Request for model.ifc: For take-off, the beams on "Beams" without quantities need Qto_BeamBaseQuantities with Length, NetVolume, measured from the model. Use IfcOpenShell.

First a look at what the model holds.

```python
import ifcopenshell
import ifcopenshell.util.element
import ifcopenshell.util.unit

model = ifcopenshell.open("model.ifc")
print(model.schema)
for unit_type in ("LENGTHUNIT", "AREAUNIT", "VOLUMEUNIT"):
    print(unit_type, ifcopenshell.util.unit.calculate_unit_scale(model, unit_type))
storey = next(s for s in model.by_type("IfcBuildingStorey") if s.Name == "Beams")
beams = [e for e in ifcopenshell.util.element.get_decomposition(storey) if e.is_a("IfcBeam")]
for e in sorted(beams, key=lambda e: e.id()):
    print(e.id(), e.is_a(), e.Name, list(ifcopenshell.util.element.get_psets(e, qtos_only=True)), sep=" | ")
```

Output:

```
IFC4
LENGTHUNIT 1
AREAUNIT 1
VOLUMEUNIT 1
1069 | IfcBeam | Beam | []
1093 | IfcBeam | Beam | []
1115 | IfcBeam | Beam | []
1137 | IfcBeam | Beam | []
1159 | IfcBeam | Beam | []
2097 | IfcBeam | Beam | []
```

```python
import ifcopenshell
import ifcopenshell.api.pset
import ifcopenshell.geom
import ifcopenshell.util.element
import ifcopenshell.util.shape
import ifcopenshell.util.unit

model = ifcopenshell.open("model.ifc")
unit_scale = ifcopenshell.util.unit.calculate_unit_scale(model)
volume_scale = ifcopenshell.util.unit.calculate_unit_scale(model, "VOLUMEUNIT")
settings = ifcopenshell.geom.settings()

storey = next(s for s in model.by_type("IfcBuildingStorey") if s.Name == "Beams")
beams = [e for e in ifcopenshell.util.element.get_decomposition(storey) if e.is_a("IfcBeam")]

for e in sorted(beams, key=lambda e: e.id()):
    if ifcopenshell.util.element.get_psets(e, qtos_only=True, should_inherit=False):
        continue
    # Geometry comes back in metres, in the element's own axes.
    shape = ifcopenshell.geom.create_shape(settings, e)
    values = {
        "Length": ifcopenshell.util.shape.get_max_xyz(shape.geometry) / unit_scale,
        "NetVolume": ifcopenshell.util.shape.get_volume(shape.geometry) / volume_scale,
    }
    qto = ifcopenshell.api.pset.add_qto(model, product=e, name="Qto_BeamBaseQuantities")
    ifcopenshell.api.pset.edit_qto(model, qto=qto, properties=values)
    print(e.id(), {k: round(v, 3) for k, v in values.items()})

model.write("model_v2.ifc")
```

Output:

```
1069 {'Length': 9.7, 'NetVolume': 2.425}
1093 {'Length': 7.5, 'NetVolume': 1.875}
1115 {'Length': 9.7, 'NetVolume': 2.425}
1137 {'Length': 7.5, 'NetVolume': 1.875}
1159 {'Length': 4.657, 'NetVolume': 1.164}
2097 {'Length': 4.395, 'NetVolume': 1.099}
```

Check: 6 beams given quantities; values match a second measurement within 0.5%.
